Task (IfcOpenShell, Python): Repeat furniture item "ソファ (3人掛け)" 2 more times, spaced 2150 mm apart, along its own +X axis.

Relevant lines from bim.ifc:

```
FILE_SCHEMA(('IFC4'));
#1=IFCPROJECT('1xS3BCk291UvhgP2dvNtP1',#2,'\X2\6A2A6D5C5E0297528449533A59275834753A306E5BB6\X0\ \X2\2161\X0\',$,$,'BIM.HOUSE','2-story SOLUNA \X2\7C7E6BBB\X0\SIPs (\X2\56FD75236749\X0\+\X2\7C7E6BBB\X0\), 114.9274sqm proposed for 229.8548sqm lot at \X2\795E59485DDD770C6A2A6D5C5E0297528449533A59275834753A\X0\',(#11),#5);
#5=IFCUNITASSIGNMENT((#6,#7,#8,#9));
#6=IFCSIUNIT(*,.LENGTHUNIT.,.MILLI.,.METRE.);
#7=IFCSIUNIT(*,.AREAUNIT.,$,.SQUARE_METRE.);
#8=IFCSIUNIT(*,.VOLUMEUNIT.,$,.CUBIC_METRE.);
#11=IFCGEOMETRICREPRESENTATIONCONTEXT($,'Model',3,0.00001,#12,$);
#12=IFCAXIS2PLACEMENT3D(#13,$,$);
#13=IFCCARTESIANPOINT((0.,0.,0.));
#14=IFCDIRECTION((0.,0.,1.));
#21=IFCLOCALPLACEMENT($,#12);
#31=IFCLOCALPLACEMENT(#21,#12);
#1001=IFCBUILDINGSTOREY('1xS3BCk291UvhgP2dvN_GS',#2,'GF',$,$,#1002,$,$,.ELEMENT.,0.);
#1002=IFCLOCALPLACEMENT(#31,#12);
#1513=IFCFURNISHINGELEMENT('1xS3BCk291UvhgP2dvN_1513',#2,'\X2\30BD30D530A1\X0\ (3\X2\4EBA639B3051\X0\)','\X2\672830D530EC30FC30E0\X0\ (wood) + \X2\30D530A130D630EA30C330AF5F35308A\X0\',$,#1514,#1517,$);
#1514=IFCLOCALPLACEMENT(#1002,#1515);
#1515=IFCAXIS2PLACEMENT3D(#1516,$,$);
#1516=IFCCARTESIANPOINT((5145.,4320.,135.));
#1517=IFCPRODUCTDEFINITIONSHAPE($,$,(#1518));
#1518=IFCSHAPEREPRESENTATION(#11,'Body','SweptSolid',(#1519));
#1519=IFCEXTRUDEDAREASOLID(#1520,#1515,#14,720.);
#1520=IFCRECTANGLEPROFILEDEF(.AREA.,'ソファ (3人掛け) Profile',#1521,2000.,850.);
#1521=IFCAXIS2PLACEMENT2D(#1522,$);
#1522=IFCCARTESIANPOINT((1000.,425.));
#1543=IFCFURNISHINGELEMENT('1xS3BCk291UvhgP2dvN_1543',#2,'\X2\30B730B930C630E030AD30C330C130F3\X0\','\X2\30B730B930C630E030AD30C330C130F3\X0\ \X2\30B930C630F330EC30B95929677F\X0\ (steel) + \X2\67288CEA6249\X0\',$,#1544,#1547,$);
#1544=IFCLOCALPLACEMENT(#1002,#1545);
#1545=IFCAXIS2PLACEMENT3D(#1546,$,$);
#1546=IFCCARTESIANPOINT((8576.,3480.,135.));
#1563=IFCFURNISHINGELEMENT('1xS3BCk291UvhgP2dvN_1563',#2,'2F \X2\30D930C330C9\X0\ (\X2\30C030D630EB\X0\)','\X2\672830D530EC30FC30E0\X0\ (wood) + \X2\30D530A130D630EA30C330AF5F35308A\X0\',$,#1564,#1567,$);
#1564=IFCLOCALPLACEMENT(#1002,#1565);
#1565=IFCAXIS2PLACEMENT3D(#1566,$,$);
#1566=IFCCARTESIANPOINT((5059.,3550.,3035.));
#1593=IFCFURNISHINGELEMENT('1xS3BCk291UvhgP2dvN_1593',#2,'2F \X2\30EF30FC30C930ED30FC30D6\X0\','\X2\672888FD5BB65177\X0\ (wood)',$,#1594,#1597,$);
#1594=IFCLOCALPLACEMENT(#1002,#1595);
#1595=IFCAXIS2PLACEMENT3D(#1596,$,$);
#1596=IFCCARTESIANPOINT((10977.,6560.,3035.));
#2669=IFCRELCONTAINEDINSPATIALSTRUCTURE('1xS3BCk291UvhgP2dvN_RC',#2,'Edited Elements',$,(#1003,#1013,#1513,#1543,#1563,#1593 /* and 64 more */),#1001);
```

```python
import ifcopenshell
import ifcopenshell.api.geometry
import ifcopenshell.api.root
import ifcopenshell.util.element
import ifcopenshell.util.placement

model = ifcopenshell.open("bim.ifc")


def reuse_history(source, copy):
    """copy_class also copies each property set's owner history, people and application; keep the originals."""
    for rel in copy.IsDefinedBy:
        if rel.is_a("IfcRelDefinesByProperties") and (history := rel.RelatingPropertyDefinition.OwnerHistory):
            rel.RelatingPropertyDefinition.OwnerHistory = source.OwnerHistory
            ifcopenshell.util.element.remove_deep2(model, history)


source = model.by_guid("1xS3BCk291UvhgP2dvN_1513")
base = ifcopenshell.util.placement.get_local_placement(source.ObjectPlacement)
step = base[:3, 0] * 2150.0

for i in range(1, 3):
    copy = ifcopenshell.api.root.copy_class(model, product=source)
    copy.Representation = ifcopenshell.util.element.copy_deep(
        model, source.Representation, exclude=["IfcGeometricRepresentationContext", "IfcRepresentationMap"]
    )
    reuse_history(source, copy)
    matrix = base.copy()
    matrix[:3, 3] += i * step
    print("added at", matrix[:3, 3].round(3) + 0.0)
    ifcopenshell.api.geometry.edit_object_placement(model, product=copy, matrix=matrix, is_si=False)

model.write("bim_updated.ifc")
```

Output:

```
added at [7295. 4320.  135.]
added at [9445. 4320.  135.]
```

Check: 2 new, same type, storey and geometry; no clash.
